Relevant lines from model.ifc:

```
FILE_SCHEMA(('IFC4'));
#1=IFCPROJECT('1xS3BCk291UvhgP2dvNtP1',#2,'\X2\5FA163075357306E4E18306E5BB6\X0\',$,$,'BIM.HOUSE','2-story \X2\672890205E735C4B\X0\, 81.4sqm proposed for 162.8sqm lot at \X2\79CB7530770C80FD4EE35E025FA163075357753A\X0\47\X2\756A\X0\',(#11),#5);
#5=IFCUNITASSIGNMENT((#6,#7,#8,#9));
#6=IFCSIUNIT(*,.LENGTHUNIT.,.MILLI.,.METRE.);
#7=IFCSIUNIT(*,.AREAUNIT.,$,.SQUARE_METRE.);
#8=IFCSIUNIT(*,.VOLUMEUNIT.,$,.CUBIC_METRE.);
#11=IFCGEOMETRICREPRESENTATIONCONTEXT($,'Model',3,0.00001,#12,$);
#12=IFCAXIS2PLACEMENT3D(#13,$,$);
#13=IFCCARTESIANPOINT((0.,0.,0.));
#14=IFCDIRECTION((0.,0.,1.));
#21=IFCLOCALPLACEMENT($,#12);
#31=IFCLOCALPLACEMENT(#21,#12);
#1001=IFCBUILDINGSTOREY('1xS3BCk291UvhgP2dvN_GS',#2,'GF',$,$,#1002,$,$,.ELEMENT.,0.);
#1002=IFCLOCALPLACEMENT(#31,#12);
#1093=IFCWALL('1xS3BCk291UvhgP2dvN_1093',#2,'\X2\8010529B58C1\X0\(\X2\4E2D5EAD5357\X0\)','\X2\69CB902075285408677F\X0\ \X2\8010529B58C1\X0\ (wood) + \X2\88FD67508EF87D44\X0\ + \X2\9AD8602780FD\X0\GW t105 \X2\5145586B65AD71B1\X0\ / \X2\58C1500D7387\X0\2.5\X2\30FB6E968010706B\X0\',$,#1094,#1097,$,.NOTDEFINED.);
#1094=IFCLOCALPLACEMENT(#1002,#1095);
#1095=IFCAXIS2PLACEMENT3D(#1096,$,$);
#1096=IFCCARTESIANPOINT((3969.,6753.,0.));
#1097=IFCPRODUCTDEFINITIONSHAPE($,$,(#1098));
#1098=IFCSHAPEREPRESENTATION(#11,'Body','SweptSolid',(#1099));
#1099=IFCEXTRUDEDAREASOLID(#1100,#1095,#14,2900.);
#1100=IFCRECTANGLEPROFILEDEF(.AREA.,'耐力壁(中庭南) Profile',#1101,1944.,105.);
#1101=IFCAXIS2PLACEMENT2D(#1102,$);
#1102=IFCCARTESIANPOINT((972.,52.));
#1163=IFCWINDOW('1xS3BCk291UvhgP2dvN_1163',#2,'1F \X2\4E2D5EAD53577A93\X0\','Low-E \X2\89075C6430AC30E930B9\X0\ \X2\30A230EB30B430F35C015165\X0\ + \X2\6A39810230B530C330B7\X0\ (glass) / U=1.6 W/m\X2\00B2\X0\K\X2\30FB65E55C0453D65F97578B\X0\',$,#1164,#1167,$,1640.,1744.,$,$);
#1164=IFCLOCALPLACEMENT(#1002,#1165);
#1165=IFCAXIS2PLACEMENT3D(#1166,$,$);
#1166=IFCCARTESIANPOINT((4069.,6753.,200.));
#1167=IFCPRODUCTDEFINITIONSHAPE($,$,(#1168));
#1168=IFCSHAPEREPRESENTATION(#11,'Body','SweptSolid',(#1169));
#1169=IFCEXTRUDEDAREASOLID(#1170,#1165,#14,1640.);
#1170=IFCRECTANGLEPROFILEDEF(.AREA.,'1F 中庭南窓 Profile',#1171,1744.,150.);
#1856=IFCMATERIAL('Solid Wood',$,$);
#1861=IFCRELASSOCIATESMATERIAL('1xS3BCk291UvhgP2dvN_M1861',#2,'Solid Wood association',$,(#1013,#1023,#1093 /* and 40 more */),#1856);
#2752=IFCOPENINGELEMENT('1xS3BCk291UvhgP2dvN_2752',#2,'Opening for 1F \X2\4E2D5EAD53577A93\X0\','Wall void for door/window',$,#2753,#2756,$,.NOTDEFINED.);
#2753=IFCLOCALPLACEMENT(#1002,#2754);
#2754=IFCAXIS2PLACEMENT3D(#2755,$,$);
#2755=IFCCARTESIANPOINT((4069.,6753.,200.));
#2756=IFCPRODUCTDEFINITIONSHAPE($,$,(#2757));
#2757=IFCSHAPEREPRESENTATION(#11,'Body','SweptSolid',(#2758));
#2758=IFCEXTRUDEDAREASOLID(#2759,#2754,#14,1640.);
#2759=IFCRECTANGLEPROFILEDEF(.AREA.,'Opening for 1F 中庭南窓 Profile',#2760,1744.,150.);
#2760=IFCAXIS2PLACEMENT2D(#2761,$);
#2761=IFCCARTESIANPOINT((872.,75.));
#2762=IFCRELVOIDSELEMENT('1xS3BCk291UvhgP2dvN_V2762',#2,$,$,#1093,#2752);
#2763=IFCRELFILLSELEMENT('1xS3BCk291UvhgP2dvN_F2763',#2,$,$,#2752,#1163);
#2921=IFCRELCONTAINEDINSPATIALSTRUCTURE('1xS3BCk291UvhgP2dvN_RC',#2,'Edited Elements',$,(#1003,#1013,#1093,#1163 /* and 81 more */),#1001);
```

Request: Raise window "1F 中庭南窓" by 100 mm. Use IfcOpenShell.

```python
import numpy as np
import ifcopenshell
import ifcopenshell.api.geometry
import ifcopenshell.util.placement
import ifcopenshell.util.unit

model = ifcopenshell.open("model.ifc")
unit_scale = ifcopenshell.util.unit.calculate_unit_scale(model)

window = model.by_id(1163)
opening = window.FillsVoids[0].RelatingOpeningElement
dz = 0.1 / unit_scale

shift = np.array([0.0, 0.0, dz])
# The window is not placed relative to its opening, so move both.
for product in (opening, window):
    matrix = ifcopenshell.util.placement.get_local_placement(product.ObjectPlacement)
    matrix[:3, 3] += shift
    ifcopenshell.api.geometry.edit_object_placement(model, product=product, matrix=matrix, is_si=False)

print(f"moved by {dz * unit_scale:+.3f} m")

model.write("model_edited.ifc")
```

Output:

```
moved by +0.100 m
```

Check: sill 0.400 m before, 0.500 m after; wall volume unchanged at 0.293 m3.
